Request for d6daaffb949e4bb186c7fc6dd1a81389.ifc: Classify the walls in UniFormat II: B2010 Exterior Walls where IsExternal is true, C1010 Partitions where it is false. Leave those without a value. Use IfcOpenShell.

First a look at what the model holds.

```python
import ifcopenshell
import ifcopenshell.util.element

model = ifcopenshell.open("d6daaffb949e4bb186c7fc6dd1a81389.ifc")
print(model.schema)
print("classifications:", [c.Name for c in model.by_type("IfcClassification")])
values = [ifcopenshell.util.element.get_pset(e, "Pset_WallCommon", "IsExternal") for e in model.by_type("IfcWall")]
for value in (True, False, None):
    print("IsExternal", value, values.count(value))
```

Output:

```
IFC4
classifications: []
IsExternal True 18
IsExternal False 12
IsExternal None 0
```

```python
import ifcopenshell
import ifcopenshell.api.classification
import ifcopenshell.util.element

model = ifcopenshell.open("d6daaffb949e4bb186c7fc6dd1a81389.ifc")

system = ifcopenshell.api.classification.add_classification(model, classification="UniFormat II")

walls = model.by_type("IfcWall")
external = {e: ifcopenshell.util.element.get_pset(e, "Pset_WallCommon", "IsExternal") for e in walls}
for flag, code, name in ((True, "B2010", "Exterior Walls"), (False, "C1010", "Partitions")):
    products = [e for e in walls if external[e] is flag]
    ifcopenshell.api.classification.add_reference(
        model, products=products, classification=system, identification=code, name=name
    )
    print(code, len(products))

model.write("d6daaffb949e4bb186c7fc6dd1a81389-out.ifc")
```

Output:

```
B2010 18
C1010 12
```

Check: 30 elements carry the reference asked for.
